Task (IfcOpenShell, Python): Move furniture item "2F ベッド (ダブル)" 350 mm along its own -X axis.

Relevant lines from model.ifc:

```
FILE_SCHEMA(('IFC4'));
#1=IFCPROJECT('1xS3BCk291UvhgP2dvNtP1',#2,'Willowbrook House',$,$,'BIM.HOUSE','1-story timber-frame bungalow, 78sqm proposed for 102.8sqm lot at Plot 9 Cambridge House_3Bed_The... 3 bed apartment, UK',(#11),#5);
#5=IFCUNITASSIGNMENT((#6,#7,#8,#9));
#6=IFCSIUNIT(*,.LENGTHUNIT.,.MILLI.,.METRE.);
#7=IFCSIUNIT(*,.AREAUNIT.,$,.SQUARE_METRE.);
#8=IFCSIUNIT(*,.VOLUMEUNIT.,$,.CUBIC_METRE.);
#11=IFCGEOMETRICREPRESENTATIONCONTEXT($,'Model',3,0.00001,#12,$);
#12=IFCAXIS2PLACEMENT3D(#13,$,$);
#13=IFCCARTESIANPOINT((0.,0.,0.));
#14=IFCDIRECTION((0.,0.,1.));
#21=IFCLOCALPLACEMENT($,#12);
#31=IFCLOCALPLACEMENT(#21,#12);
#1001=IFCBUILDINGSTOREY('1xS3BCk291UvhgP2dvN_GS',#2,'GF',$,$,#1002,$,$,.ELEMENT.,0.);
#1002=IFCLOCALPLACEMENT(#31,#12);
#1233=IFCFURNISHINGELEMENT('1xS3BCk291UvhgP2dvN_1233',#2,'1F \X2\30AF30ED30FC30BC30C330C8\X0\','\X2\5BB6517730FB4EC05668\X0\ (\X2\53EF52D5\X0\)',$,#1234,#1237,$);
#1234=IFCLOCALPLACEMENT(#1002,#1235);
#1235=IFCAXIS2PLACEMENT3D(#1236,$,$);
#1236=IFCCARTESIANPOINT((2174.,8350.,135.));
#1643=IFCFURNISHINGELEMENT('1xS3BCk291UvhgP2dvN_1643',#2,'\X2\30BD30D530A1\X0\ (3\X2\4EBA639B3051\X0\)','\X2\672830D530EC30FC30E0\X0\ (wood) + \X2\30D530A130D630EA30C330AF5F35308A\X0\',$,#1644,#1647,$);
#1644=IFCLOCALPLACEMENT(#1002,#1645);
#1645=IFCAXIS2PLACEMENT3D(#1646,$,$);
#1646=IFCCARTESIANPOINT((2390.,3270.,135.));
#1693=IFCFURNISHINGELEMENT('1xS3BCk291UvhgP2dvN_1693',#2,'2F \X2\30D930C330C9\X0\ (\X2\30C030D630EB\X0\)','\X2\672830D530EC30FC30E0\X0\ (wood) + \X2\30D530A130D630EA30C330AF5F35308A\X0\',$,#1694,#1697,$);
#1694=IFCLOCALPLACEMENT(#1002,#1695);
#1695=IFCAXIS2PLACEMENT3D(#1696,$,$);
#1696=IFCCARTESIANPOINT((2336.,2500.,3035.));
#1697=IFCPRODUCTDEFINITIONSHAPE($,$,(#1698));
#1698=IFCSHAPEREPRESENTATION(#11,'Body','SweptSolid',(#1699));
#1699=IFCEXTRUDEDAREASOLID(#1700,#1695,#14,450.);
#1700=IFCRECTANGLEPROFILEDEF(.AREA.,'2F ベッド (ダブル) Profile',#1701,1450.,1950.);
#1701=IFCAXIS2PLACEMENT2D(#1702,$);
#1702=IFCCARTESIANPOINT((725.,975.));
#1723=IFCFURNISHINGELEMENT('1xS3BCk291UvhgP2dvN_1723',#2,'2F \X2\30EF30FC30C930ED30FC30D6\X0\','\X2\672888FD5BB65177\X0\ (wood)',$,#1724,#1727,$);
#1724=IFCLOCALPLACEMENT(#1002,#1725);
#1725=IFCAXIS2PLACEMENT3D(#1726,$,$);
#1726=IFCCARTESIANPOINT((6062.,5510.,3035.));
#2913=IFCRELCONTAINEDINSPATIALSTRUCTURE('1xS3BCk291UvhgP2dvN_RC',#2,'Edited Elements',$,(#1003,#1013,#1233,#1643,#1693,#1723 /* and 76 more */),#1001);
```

```python
import ifcopenshell
import ifcopenshell.api.geometry
import ifcopenshell.util.placement
import ifcopenshell.util.unit

model = ifcopenshell.open("model.ifc")
unit_scale = ifcopenshell.util.unit.calculate_unit_scale(model)

item = model.by_id(1693)
matrix = ifcopenshell.util.placement.get_local_placement(item.ObjectPlacement)
matrix[:3, 3] -= matrix[:3, 0] * 0.35 / unit_scale
ifcopenshell.api.geometry.edit_object_placement(model, product=item, matrix=matrix, is_si=False)

print(ifcopenshell.util.placement.get_local_placement(item.ObjectPlacement).round(3) + 0.0)

model.write("model_v2.ifc")
```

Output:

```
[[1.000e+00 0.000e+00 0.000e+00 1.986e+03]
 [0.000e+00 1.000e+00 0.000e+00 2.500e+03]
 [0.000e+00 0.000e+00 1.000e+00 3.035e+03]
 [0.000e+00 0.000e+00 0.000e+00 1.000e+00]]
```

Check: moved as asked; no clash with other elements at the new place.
